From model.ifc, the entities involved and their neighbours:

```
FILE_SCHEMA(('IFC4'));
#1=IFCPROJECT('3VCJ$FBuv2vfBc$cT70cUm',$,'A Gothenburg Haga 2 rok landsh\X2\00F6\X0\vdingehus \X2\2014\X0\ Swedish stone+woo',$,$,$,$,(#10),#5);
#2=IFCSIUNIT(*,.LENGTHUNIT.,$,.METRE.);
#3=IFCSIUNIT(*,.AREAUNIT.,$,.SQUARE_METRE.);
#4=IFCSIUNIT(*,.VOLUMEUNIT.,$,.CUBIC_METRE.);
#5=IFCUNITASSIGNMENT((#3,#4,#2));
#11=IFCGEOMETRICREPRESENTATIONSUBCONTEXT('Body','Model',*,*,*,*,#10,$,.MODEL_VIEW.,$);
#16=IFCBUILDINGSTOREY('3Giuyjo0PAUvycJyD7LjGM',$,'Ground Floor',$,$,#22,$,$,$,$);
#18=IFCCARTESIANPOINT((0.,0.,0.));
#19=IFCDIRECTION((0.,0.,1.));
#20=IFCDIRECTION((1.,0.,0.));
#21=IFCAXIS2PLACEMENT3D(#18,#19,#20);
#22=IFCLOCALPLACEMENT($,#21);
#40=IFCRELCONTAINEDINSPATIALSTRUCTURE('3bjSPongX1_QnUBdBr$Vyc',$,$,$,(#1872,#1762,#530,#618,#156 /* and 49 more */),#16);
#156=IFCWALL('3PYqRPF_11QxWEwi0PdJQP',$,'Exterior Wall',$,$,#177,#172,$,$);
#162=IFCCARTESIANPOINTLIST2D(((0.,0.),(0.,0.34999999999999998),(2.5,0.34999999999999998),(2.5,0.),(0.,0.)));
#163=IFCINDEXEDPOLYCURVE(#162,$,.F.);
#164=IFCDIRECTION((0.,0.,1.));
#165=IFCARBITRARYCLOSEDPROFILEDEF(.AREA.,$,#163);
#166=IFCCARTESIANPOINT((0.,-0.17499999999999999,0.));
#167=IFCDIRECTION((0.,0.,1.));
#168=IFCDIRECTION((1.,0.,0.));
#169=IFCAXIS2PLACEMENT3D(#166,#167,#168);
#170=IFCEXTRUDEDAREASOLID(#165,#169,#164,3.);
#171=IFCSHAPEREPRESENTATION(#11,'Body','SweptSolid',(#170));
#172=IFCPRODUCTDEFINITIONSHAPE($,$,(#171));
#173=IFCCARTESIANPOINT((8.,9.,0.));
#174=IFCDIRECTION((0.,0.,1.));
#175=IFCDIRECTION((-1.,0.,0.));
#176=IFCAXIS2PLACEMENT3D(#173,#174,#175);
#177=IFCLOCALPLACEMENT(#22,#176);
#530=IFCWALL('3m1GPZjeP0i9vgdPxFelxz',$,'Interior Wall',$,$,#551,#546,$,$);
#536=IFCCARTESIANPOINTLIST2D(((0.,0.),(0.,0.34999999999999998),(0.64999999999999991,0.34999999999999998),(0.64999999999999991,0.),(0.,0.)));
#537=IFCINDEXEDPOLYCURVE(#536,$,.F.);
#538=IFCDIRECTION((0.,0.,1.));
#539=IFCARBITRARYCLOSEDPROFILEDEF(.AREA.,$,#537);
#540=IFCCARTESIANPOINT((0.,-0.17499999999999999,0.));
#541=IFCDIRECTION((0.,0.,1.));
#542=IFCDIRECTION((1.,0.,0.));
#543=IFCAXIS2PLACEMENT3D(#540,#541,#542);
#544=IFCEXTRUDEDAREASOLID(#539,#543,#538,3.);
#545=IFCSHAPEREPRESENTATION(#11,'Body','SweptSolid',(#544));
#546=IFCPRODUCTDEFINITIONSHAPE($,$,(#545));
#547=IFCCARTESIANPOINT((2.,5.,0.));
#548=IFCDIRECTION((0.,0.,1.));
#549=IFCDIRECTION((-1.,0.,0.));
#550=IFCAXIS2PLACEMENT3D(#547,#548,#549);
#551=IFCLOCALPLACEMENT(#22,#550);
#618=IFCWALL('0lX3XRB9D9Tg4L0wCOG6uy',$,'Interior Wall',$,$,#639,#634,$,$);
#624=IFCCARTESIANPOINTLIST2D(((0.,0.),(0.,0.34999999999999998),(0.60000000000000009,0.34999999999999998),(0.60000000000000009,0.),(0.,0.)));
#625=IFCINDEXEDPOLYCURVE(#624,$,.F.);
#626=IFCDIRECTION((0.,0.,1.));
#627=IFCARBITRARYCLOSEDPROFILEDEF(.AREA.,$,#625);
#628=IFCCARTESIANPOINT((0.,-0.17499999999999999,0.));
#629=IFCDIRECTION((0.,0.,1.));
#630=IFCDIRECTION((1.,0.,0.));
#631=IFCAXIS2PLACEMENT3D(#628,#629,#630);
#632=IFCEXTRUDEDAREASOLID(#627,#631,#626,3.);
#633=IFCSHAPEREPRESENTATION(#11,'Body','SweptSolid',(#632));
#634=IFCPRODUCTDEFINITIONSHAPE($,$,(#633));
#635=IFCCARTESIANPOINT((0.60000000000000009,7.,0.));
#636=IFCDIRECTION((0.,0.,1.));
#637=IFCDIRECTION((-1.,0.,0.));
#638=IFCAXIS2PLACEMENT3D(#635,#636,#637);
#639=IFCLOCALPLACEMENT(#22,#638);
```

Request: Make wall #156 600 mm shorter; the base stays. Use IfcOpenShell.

```python
import ifcopenshell
import ifcopenshell.geom
import ifcopenshell.util.representation
import ifcopenshell.util.shape
import ifcopenshell.util.unit

model = ifcopenshell.open("model.ifc")
unit_scale = ifcopenshell.util.unit.calculate_unit_scale(model)
settings = ifcopenshell.geom.settings()


def volume(element):
    """Net volume in cubic metres, openings subtracted."""
    shape = ifcopenshell.geom.create_shape(settings, element)
    return ifcopenshell.util.shape.get_volume(shape.geometry)


wall = model.by_guid("3PYqRPF_11QxWEwi0PdJQP")
before = volume(wall)

body = ifcopenshell.util.representation.get_representation(wall, "Model", "Body")
solid = body.Items[0]
old_height = solid.Depth
solid.Depth -= 0.6 / unit_scale
after = volume(wall)

print(f"height {old_height:g} -> {solid.Depth:g}, volume {before:.3f} -> {after:.3f} m3")

model.write("model_edited.ifc")
```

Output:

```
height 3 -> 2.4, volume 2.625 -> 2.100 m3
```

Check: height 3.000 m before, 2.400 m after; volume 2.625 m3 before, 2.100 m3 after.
